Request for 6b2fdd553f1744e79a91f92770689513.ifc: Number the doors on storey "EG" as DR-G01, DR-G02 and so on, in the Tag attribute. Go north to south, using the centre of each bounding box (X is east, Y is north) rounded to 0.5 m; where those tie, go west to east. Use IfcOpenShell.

First a look at what the model holds.

```python
import ifcopenshell
import ifcopenshell.util.element
import ifcopenshell.util.placement

model = ifcopenshell.open("6b2fdd553f1744e79a91f92770689513.ifc")
print(model.schema)
storey = next(s for s in model.by_type("IfcBuildingStorey") if s.Name == "EG")
doors = [e for e in ifcopenshell.util.element.get_decomposition(storey) if e.is_a("IfcDoor")]
for e in sorted(doors, key=lambda e: e.id()):
    origin = ifcopenshell.util.placement.get_local_placement(e.ObjectPlacement)[:3, 3]
    print(e.id(), e.Tag, e.Name, origin.round(2) + 0.0, sep=" | ")
```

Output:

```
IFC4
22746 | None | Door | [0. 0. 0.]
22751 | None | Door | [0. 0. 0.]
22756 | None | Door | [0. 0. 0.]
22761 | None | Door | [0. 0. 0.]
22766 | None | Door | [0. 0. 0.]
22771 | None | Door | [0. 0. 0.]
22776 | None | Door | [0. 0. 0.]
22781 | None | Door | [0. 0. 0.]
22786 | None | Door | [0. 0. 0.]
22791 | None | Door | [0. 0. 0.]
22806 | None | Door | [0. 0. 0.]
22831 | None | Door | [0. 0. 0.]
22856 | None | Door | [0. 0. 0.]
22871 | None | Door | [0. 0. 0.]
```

```python
import ifcopenshell
import ifcopenshell.geom
import ifcopenshell.util.element
import ifcopenshell.util.shape

model = ifcopenshell.open("6b2fdd553f1744e79a91f92770689513.ifc")
settings = ifcopenshell.geom.settings()
settings.set("use-world-coords", True)


def centre(element):
    shape = ifcopenshell.geom.create_shape(settings, element)
    return ifcopenshell.util.shape.get_bbox_centroid(shape.geometry)


storey = next(s for s in model.by_type("IfcBuildingStorey") if s.Name == "EG")
doors = [e for e in ifcopenshell.util.element.get_decomposition(storey) if e.is_a("IfcDoor")]

# Insertion points can sit at a corner or the storey origin, so sort by the geometry (in metres).
centres = {e: centre(e) for e in doors}
doors.sort(key=lambda e: (-round(centres[e][1] / 0.5), centres[e][0]))

for i, e in enumerate(doors, start=1):
    number = f"DR-G{i:02d}"
    e.Tag = number
    print(e.id(), number)

model.write("6b2fdd553f1744e79a91f92770689513_edited.ifc")
```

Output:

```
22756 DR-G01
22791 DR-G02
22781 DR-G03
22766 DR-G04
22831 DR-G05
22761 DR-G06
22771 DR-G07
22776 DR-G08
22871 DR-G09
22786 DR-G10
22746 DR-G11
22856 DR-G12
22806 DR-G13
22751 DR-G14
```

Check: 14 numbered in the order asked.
